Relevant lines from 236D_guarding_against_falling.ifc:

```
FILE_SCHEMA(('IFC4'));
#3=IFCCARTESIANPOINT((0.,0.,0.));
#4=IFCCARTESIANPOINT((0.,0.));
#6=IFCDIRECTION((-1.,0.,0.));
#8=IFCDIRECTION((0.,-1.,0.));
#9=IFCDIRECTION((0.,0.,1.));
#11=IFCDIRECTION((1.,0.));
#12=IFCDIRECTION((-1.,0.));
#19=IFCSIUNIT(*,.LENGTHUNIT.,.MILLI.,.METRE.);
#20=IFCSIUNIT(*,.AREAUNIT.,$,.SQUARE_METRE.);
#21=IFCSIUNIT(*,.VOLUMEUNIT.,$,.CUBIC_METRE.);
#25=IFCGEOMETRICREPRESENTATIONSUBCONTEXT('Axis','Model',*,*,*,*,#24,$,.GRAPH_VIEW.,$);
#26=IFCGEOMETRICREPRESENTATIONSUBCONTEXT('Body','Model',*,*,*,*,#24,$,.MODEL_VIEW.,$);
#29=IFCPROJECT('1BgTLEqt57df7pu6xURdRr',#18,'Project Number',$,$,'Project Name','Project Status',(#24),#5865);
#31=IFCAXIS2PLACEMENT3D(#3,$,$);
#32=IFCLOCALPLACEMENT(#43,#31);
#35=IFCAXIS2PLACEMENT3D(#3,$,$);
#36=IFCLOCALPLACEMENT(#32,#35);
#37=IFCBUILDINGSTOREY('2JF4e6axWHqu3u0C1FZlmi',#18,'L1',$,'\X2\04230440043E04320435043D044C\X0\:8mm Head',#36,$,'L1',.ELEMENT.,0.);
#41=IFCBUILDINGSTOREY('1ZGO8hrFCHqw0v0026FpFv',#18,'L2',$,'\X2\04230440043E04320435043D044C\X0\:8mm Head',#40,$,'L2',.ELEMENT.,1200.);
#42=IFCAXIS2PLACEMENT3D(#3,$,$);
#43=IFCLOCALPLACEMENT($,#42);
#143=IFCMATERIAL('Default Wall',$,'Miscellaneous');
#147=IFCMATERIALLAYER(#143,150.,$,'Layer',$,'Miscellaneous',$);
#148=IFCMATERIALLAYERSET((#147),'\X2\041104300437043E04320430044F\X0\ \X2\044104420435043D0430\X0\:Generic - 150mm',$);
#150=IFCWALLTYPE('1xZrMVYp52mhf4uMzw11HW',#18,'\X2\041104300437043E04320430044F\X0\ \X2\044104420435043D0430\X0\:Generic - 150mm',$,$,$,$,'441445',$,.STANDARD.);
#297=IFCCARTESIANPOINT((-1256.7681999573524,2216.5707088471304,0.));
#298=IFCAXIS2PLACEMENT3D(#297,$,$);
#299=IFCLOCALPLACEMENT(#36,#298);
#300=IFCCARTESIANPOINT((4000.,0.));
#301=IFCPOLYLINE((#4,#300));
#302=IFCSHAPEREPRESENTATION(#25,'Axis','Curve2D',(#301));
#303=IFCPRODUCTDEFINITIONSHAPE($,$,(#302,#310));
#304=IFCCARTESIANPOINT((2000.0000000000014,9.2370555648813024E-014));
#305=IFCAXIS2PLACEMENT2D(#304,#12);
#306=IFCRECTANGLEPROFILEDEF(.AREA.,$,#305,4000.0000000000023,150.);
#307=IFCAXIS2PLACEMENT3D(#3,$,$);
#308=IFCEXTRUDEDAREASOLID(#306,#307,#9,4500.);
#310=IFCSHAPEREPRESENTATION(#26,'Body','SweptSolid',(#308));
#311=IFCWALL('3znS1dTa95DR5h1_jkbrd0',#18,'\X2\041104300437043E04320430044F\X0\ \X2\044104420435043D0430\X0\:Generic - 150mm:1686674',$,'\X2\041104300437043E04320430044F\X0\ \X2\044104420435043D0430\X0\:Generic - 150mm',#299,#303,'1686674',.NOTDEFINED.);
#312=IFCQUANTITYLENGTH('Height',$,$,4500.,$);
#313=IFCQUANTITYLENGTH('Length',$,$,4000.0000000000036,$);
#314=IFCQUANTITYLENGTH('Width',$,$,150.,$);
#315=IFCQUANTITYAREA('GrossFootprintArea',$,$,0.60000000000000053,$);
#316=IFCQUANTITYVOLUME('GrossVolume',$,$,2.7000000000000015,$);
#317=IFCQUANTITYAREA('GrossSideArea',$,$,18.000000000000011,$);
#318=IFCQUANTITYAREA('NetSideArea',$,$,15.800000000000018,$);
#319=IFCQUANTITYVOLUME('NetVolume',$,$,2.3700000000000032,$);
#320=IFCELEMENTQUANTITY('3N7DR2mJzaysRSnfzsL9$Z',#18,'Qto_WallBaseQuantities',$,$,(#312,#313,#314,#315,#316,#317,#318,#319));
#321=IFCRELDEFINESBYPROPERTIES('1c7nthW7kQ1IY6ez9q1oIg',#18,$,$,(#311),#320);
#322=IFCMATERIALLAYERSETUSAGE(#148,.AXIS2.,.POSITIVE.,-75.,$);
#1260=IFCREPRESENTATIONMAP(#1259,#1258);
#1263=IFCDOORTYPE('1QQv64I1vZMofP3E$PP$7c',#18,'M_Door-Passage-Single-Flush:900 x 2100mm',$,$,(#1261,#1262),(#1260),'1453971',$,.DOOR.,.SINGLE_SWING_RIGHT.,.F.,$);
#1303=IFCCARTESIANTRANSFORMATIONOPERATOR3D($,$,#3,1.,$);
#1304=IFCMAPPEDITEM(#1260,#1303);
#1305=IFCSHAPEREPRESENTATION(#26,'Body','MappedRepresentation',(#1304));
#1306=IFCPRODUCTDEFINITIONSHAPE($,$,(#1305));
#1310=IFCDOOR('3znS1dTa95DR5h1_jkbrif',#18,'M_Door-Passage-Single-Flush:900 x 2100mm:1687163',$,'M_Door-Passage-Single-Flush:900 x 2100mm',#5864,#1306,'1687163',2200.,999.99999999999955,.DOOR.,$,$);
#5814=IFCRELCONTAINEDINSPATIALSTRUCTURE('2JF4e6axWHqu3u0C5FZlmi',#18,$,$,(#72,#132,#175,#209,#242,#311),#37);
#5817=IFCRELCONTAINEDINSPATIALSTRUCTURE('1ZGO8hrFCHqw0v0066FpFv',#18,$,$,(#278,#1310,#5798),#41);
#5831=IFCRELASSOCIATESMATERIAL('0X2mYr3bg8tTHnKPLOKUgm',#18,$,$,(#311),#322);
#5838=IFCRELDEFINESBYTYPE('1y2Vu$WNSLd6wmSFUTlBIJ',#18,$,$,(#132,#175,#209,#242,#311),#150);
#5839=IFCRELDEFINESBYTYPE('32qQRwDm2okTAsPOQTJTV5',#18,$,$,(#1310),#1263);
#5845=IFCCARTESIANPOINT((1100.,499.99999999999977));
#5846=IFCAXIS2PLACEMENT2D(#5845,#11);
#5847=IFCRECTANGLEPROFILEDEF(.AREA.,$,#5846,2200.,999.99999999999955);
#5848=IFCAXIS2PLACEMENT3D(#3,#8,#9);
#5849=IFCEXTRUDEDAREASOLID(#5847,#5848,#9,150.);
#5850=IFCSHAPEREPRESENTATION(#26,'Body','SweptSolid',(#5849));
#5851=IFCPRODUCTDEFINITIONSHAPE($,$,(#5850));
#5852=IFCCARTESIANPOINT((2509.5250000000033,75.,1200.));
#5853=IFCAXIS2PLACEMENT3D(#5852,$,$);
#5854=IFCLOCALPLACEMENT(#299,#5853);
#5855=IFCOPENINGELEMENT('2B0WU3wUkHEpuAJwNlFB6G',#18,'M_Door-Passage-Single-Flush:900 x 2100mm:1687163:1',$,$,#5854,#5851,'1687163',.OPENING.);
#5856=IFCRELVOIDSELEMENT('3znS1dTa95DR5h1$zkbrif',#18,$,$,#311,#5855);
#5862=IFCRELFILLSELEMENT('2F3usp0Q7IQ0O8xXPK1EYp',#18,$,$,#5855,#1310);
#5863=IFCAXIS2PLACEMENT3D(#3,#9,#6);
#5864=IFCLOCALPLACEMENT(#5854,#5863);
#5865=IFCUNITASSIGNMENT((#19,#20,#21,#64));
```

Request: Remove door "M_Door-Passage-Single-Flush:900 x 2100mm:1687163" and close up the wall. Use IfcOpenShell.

```python
import ifcopenshell
import ifcopenshell.api.feature
import ifcopenshell.api.pset
import ifcopenshell.api.root
import ifcopenshell.geom
import ifcopenshell.util.element
import ifcopenshell.util.shape
import ifcopenshell.util.unit

model = ifcopenshell.open("236D_guarding_against_falling.ifc")
area_scale = ifcopenshell.util.unit.calculate_unit_scale(model, "AREAUNIT")
volume_scale = ifcopenshell.util.unit.calculate_unit_scale(model, "VOLUMEUNIT")
settings = ifcopenshell.geom.settings()


def volume(element):
    """Net volume in cubic metres, openings subtracted."""
    shape = ifcopenshell.geom.create_shape(settings, element)
    return ifcopenshell.util.shape.get_volume(shape.geometry)


door = model.by_id(1310)
opening = door.FillsVoids[0].RelatingOpeningElement
wall = opening.VoidsElements[0].RelatingBuildingElement
before = volume(wall)

ifcopenshell.api.root.remove_product(model, product=door)
ifcopenshell.api.feature.remove_feature(model, feature=opening)

after = volume(wall)
thickness = 0.15  # wall thickness in metres

# Update the wall's stored quantities.
qto = model.by_id(ifcopenshell.util.element.get_pset(wall, "Qto_WallBaseQuantities", should_inherit=False)["id"])
ifcopenshell.api.pset.edit_qto(model, qto=qto, properties={
    "NetSideArea": after / thickness / area_scale,
    "NetVolume": after / volume_scale,
})

print(f"wall volume {before:.3f} -> {after:.3f} m3")

model.write("236D_guarding_against_falling-out.ifc")
```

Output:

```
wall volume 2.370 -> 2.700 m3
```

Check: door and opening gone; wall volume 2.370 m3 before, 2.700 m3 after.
